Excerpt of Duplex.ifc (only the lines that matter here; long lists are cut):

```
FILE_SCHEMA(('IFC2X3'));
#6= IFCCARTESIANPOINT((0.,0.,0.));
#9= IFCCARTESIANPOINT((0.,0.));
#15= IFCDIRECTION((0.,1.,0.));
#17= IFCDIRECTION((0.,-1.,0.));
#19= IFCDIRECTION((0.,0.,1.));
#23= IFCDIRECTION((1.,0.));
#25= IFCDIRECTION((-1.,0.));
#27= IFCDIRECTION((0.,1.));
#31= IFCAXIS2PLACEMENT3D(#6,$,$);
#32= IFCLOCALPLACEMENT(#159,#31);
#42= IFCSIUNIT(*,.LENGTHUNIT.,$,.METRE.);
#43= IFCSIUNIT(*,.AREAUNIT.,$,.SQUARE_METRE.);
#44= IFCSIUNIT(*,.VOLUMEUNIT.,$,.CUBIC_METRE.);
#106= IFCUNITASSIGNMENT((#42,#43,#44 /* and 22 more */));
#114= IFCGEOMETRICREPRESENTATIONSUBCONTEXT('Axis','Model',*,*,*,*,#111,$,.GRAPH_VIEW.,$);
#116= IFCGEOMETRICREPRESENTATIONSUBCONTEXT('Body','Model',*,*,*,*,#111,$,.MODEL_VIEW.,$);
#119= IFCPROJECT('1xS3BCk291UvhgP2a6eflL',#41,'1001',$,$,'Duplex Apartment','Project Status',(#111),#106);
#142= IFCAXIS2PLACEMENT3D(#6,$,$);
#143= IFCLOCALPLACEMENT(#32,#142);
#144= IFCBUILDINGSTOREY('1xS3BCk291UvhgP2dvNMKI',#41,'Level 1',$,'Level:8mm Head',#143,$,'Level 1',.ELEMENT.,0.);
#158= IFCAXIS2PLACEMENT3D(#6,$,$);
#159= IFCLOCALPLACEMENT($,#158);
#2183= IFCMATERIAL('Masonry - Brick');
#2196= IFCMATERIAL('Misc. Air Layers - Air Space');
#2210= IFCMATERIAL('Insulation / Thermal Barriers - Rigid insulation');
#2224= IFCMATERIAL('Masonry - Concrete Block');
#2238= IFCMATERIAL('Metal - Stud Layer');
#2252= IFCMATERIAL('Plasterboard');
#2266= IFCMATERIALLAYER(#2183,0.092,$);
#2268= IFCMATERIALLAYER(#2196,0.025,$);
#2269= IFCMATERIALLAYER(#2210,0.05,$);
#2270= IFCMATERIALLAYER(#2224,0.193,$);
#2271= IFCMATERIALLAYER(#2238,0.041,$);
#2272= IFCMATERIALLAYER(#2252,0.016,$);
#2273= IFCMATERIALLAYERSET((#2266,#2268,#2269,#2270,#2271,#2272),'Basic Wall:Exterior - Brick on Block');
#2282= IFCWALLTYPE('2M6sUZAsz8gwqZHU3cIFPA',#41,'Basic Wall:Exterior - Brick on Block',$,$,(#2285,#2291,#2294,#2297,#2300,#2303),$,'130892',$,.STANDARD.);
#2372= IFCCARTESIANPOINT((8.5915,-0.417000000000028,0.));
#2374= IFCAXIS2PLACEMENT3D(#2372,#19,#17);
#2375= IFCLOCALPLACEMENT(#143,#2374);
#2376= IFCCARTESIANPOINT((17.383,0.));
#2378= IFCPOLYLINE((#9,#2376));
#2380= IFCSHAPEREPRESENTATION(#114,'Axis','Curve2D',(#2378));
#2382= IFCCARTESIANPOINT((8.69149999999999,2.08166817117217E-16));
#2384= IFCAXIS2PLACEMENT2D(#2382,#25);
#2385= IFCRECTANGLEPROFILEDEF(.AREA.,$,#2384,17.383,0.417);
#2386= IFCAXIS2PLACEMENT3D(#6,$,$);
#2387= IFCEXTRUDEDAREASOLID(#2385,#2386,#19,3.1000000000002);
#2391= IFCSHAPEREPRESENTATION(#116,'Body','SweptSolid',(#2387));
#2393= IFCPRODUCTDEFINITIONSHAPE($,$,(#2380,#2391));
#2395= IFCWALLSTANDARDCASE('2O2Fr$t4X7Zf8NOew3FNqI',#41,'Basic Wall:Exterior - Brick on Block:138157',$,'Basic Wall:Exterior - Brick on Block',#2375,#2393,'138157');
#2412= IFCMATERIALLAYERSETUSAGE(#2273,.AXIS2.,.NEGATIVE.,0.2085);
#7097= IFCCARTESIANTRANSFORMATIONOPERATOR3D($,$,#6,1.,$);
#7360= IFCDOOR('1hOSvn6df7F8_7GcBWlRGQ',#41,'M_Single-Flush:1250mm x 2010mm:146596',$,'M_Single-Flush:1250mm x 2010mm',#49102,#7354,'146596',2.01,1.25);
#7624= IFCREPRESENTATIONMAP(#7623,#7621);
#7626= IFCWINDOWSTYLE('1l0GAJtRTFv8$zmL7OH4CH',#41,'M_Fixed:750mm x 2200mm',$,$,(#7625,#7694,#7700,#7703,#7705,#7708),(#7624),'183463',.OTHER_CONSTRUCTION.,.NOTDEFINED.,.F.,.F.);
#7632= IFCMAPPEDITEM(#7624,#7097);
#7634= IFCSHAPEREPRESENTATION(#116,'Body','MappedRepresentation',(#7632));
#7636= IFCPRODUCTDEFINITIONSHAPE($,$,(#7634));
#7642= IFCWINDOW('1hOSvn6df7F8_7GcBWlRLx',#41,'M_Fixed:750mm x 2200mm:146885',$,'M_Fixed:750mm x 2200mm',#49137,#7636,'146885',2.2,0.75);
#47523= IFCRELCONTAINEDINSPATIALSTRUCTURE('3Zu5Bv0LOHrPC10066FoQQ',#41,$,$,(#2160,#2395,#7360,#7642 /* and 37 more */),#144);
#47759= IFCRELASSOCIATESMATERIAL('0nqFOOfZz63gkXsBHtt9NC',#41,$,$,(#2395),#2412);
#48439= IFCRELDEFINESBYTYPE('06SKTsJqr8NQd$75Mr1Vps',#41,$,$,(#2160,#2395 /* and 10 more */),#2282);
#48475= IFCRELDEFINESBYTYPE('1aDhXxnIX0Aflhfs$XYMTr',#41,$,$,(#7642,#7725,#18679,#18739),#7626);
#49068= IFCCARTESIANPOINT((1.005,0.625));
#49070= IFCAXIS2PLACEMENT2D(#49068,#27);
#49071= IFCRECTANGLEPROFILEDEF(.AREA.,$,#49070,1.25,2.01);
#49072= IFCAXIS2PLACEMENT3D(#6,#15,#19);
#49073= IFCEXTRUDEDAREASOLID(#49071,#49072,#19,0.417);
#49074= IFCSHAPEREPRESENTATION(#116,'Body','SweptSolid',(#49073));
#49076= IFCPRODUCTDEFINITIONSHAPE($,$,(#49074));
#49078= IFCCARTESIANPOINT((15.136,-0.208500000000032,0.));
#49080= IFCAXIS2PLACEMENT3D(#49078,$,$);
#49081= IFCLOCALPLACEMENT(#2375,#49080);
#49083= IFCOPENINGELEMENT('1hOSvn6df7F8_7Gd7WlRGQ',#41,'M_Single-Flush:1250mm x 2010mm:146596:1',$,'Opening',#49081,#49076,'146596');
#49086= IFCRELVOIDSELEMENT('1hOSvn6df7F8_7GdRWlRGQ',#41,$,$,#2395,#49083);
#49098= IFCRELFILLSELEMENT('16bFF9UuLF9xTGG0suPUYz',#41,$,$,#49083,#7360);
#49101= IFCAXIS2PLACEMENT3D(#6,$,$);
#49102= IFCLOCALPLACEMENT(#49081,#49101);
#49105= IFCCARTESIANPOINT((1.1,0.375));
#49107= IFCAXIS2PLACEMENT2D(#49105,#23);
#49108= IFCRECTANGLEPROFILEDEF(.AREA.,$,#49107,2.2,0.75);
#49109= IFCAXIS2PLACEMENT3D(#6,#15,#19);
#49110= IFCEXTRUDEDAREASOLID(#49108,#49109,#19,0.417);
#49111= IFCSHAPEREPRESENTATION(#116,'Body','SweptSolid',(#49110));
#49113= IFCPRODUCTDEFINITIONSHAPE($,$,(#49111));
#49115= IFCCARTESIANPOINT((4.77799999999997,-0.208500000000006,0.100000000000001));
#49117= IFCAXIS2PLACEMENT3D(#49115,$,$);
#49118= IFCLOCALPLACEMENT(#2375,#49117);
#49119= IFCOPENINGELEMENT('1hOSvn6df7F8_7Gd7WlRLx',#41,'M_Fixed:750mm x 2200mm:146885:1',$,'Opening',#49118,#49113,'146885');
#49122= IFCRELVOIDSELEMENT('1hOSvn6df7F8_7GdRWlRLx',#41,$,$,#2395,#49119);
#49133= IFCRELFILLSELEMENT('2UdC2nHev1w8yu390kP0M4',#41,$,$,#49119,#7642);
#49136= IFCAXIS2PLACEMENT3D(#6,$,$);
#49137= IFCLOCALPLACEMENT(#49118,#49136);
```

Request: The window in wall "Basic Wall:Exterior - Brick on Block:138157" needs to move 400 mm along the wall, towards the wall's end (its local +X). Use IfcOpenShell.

```python
import ifcopenshell
import ifcopenshell.api.geometry
import ifcopenshell.util.placement

model = ifcopenshell.open("Duplex.ifc")

window = model.by_guid("1hOSvn6df7F8_7GcBWlRLx")
opening = window.FillsVoids[0].RelatingOpeningElement
wall = opening.VoidsElements[0].RelatingBuildingElement

wall_matrix = ifcopenshell.util.placement.get_local_placement(wall.ObjectPlacement)
shift = wall_matrix[:3, 0] * 0.4
before = ifcopenshell.util.placement.get_local_placement(window.ObjectPlacement)[:3, 3].copy()

# The window is placed relative to its opening, so it follows when the opening moves.
matrix = ifcopenshell.util.placement.get_local_placement(opening.ObjectPlacement)
matrix[:3, 3] += shift
ifcopenshell.api.geometry.edit_object_placement(
    model, product=opening, matrix=matrix, is_si=False, should_transform_children=True
)

after = ifcopenshell.util.placement.get_local_placement(window.ObjectPlacement)[:3, 3]
print("window moved by", (after - before).round(3) + 0.0)

model.write("Duplex_edited.ifc")
```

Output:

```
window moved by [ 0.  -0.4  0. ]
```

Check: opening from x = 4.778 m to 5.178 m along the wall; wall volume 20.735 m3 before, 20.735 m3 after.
